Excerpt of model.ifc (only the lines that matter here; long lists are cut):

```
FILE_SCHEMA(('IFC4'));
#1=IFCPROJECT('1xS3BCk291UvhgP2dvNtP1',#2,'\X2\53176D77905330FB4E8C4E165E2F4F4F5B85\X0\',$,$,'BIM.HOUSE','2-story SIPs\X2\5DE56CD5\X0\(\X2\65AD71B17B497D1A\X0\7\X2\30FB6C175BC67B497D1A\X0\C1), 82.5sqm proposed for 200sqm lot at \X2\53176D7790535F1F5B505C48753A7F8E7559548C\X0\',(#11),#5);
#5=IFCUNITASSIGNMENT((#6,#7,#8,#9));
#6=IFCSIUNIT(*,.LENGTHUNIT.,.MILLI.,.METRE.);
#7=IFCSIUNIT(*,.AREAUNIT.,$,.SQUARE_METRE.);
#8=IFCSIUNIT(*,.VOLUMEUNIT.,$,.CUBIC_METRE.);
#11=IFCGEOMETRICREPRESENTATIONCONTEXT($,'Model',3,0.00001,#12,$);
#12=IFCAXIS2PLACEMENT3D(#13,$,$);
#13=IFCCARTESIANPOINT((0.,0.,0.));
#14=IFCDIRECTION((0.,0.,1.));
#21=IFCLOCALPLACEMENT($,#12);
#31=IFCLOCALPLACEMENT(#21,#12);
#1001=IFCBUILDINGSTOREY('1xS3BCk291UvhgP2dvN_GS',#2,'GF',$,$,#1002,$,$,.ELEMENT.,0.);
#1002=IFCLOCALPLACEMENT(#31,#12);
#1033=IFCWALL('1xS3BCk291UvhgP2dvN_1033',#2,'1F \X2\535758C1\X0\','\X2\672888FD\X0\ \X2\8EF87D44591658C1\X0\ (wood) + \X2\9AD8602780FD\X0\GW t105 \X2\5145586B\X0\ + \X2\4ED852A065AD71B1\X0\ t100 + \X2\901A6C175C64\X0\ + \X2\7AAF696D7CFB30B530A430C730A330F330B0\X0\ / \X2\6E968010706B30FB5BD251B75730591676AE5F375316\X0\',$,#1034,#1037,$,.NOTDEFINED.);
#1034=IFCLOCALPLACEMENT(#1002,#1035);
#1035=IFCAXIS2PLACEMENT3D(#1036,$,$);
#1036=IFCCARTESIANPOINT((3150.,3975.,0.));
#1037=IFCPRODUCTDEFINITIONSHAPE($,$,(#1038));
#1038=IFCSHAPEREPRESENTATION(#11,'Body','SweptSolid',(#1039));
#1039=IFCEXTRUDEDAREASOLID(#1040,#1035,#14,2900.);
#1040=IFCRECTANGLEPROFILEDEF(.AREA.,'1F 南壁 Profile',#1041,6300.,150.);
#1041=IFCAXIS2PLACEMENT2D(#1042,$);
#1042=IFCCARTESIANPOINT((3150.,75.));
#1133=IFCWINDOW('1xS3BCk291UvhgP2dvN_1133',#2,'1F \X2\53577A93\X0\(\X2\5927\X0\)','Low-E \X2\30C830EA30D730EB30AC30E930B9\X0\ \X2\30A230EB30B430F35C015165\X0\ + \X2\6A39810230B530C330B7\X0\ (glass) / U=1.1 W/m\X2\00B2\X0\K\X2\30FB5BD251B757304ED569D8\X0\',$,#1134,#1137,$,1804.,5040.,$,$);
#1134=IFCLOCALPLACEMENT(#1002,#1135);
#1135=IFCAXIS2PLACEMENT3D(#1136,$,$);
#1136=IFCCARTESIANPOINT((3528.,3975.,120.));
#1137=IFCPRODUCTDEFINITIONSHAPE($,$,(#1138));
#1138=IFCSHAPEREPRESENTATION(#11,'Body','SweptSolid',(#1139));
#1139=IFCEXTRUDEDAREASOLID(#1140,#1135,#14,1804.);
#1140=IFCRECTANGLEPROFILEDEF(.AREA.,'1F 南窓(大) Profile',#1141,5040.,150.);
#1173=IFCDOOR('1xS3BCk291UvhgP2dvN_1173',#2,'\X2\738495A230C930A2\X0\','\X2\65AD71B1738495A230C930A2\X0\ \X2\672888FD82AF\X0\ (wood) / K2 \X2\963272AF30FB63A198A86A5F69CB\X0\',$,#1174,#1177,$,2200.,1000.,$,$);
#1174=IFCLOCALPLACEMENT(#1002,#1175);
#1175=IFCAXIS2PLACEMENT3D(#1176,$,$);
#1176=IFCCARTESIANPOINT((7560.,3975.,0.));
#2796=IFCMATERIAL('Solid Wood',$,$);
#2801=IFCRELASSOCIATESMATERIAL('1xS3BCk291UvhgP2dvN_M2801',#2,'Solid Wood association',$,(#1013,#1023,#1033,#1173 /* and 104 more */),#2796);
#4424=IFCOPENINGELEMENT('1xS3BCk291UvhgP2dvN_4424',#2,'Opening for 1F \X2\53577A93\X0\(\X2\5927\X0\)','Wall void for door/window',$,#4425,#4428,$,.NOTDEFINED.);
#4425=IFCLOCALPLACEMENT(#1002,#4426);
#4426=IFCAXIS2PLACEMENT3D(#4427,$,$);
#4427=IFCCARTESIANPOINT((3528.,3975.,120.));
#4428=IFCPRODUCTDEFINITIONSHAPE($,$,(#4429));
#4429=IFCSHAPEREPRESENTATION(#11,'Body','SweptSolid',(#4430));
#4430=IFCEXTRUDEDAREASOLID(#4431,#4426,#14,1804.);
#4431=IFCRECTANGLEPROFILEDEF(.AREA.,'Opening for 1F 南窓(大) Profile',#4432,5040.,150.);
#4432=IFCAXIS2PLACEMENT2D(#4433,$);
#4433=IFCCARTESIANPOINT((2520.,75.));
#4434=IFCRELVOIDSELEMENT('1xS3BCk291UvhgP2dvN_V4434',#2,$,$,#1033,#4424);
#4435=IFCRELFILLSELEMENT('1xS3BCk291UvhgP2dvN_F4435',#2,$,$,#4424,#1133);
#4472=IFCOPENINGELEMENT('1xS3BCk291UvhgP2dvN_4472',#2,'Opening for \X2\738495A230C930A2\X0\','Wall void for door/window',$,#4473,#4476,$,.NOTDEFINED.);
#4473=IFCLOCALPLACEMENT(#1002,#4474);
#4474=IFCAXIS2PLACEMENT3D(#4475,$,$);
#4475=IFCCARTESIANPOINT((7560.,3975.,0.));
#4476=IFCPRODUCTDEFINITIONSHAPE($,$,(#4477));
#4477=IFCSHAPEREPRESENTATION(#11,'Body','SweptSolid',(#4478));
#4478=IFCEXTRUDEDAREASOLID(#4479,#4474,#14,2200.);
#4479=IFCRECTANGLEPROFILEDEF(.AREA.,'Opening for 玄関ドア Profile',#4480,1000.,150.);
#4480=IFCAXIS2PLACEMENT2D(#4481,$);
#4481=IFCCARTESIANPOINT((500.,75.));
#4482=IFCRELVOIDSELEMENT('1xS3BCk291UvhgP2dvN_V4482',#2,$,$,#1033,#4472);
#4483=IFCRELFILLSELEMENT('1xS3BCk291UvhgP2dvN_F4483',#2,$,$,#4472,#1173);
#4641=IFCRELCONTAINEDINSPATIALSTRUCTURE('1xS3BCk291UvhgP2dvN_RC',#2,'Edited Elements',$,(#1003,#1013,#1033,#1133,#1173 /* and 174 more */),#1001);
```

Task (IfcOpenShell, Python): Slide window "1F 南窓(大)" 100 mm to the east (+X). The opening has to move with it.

```python
import ifcopenshell
import ifcopenshell.api.geometry
import ifcopenshell.util.placement

model = ifcopenshell.open("model.ifc")

window = model.by_guid("1xS3BCk291UvhgP2dvN_1133")
opening = window.FillsVoids[0].RelatingOpeningElement
wall = opening.VoidsElements[0].RelatingBuildingElement

wall_matrix = ifcopenshell.util.placement.get_local_placement(wall.ObjectPlacement)
shift = wall_matrix[:3, 0] * 100.0
before = ifcopenshell.util.placement.get_local_placement(window.ObjectPlacement)[:3, 3].copy()

# The window is not placed relative to its opening, so move both.
for product in (opening, window):
    matrix = ifcopenshell.util.placement.get_local_placement(product.ObjectPlacement)
    matrix[:3, 3] += shift
    ifcopenshell.api.geometry.edit_object_placement(model, product=product, matrix=matrix, is_si=False)

after = ifcopenshell.util.placement.get_local_placement(window.ObjectPlacement)[:3, 3]
print("window moved by", (after - before).round(3) + 0.0)

model.write("model_rev.ifc")
```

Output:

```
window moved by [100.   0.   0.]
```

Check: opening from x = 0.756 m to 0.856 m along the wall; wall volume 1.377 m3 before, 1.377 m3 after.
